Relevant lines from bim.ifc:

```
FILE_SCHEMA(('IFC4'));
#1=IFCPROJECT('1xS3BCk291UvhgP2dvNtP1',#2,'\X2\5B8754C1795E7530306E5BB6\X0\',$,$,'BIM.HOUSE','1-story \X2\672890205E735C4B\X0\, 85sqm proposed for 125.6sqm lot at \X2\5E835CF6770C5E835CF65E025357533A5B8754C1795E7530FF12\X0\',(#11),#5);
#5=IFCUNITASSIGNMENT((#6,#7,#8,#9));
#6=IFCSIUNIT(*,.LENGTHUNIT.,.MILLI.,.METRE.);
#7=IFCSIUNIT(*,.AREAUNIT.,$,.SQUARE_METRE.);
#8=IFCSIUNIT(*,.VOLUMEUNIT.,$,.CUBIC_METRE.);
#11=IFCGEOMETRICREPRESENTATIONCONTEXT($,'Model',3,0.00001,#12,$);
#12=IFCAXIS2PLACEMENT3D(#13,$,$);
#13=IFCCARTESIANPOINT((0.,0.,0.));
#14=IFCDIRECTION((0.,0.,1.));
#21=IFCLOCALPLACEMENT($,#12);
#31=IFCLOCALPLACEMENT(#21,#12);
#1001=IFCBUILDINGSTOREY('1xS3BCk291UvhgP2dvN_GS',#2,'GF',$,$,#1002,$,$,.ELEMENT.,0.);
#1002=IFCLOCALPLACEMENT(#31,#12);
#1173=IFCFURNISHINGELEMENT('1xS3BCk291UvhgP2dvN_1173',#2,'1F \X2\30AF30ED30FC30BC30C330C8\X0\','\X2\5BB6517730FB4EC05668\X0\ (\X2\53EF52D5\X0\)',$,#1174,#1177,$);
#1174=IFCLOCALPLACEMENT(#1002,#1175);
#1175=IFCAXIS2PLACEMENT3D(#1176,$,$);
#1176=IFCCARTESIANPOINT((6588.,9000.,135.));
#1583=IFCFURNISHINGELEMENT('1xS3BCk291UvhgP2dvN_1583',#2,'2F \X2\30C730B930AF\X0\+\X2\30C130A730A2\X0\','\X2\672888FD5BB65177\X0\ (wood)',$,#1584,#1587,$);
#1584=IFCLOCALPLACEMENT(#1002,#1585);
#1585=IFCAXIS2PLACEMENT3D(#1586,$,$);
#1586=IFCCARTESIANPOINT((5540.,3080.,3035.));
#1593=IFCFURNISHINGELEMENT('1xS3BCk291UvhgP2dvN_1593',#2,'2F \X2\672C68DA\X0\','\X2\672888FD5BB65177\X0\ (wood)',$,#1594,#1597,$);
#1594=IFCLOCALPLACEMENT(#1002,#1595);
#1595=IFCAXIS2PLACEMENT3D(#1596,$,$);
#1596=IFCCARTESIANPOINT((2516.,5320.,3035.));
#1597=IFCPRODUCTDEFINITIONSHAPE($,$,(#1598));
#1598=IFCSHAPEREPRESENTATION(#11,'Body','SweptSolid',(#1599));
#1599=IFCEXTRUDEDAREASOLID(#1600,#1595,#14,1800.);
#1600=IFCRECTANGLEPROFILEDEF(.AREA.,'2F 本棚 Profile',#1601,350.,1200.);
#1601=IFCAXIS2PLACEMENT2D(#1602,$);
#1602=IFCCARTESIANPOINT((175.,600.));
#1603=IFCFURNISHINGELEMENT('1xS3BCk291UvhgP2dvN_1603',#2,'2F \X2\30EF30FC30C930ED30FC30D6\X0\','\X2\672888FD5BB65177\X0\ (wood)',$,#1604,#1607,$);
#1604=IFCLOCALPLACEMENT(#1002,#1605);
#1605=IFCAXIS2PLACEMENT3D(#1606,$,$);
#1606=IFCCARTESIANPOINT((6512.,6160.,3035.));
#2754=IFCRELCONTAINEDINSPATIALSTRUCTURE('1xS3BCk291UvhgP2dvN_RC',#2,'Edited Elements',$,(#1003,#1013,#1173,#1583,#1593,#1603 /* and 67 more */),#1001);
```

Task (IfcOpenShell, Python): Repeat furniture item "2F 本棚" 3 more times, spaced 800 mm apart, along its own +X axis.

```python
import ifcopenshell
import ifcopenshell.api.geometry
import ifcopenshell.api.root
import ifcopenshell.util.element
import ifcopenshell.util.placement
import ifcopenshell.util.unit

model = ifcopenshell.open("bim.ifc")
unit_scale = ifcopenshell.util.unit.calculate_unit_scale(model)


def reuse_history(source, copy):
    """copy_class also copies each property set's owner history, people and application; keep the originals."""
    for rel in copy.IsDefinedBy:
        if rel.is_a("IfcRelDefinesByProperties") and (history := rel.RelatingPropertyDefinition.OwnerHistory):
            rel.RelatingPropertyDefinition.OwnerHistory = source.OwnerHistory
            ifcopenshell.util.element.remove_deep2(model, history)


source = model.by_id(1593)
base = ifcopenshell.util.placement.get_local_placement(source.ObjectPlacement)
step = base[:3, 0] * 0.8 / unit_scale

for i in range(1, 4):
    copy = ifcopenshell.api.root.copy_class(model, product=source)
    copy.Representation = ifcopenshell.util.element.copy_deep(
        model, source.Representation, exclude=["IfcGeometricRepresentationContext", "IfcRepresentationMap"]
    )
    reuse_history(source, copy)
    matrix = base.copy()
    matrix[:3, 3] += i * step
    print("added at", matrix[:3, 3].round(3) + 0.0)
    ifcopenshell.api.geometry.edit_object_placement(model, product=copy, matrix=matrix, is_si=False)

model.write("bim_edited.ifc")
```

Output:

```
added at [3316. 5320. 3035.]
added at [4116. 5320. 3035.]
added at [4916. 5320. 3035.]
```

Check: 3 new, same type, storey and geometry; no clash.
